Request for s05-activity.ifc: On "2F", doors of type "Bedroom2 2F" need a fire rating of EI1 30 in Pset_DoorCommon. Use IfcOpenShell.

First a look at what the model holds.

```python
import ifcopenshell
import ifcopenshell.util.element

model = ifcopenshell.open("s05-activity.ifc")
print(model.schema)
storey = next(s for s in model.by_type("IfcBuildingStorey") if s.Name == "2F")
doors = [e for e in ifcopenshell.util.element.get_decomposition(storey) if e.is_a("IfcDoor")]
seen = {}
for e in doors:
    element_type = ifcopenshell.util.element.get_type(e)
    key = (element_type.Name if element_type != e and element_type else None, ifcopenshell.util.element.get_pset(e, "Pset_DoorCommon", "FireRating"))
    seen[key] = seen.get(key, 0) + 1
for (name, value), count in sorted(seen.items(), key=str):
    print(count, "x", name, "|", value)
```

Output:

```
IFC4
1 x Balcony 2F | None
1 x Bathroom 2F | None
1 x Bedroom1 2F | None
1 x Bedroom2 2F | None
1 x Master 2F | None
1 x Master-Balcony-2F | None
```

```python
import ifcopenshell
import ifcopenshell.api.pset
import ifcopenshell.util.element

model = ifcopenshell.open("s05-activity.ifc")

storey = next(s for s in model.by_type("IfcBuildingStorey") if s.Name == "2F")
doors = [e for e in ifcopenshell.util.element.get_decomposition(storey) if e.is_a("IfcDoor")]

count = 0
for e in doors:
    element_type = ifcopenshell.util.element.get_type(e)
    if element_type in (None, e) or element_type.Name != "Bedroom2 2F":
        continue
    # add_pset returns the element's existing set when there is one.
    pset = ifcopenshell.api.pset.add_pset(model, product=e, name="Pset_DoorCommon")
    ifcopenshell.api.pset.edit_pset(model, pset=pset, properties={"FireRating": "EI1 30"})
    count += 1

print(count, "doors updated")

model.write("s05-activity_edited.ifc")
```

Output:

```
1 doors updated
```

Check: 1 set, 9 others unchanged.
